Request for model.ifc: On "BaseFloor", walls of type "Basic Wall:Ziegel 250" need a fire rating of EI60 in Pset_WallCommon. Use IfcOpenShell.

First a look at what the model holds.

```python
import ifcopenshell
import ifcopenshell.util.element

model = ifcopenshell.open("model.ifc")
print(model.schema)
storey = next(s for s in model.by_type("IfcBuildingStorey") if s.Name == "BaseFloor")
walls = [e for e in ifcopenshell.util.element.get_decomposition(storey) if e.is_a("IfcWall")]
seen = {}
for e in walls:
    element_type = ifcopenshell.util.element.get_type(e)
    key = (element_type.Name if element_type != e and element_type else None, ifcopenshell.util.element.get_pset(e, "Pset_WallCommon", "FireRating"))
    seen[key] = seen.get(key, 0) + 1
for (name, value), count in sorted(seen.items(), key=str):
    print(count, "x", name, "|", value)
```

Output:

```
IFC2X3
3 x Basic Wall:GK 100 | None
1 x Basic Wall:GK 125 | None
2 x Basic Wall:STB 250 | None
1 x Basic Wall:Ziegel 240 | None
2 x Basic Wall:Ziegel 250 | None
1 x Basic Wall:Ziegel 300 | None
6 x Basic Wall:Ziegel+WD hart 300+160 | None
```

```python
import ifcopenshell
import ifcopenshell.api.pset
import ifcopenshell.util.element

model = ifcopenshell.open("model.ifc")

storey = next(s for s in model.by_type("IfcBuildingStorey") if s.Name == "BaseFloor")
walls = [e for e in ifcopenshell.util.element.get_decomposition(storey) if e.is_a("IfcWall")]

count = 0
for e in walls:
    element_type = ifcopenshell.util.element.get_type(e)
    if element_type in (None, e) or element_type.Name != "Basic Wall:Ziegel 250":
        continue
    # add_pset returns the element's existing set when there is one.
    pset = ifcopenshell.api.pset.add_pset(model, product=e, name="Pset_WallCommon")
    ifcopenshell.api.pset.edit_pset(model, pset=pset, properties={"FireRating": "EI60"})
    count += 1

print(count, "walls updated")

model.write("model_rev.ifc")
```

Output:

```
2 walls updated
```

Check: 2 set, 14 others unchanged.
